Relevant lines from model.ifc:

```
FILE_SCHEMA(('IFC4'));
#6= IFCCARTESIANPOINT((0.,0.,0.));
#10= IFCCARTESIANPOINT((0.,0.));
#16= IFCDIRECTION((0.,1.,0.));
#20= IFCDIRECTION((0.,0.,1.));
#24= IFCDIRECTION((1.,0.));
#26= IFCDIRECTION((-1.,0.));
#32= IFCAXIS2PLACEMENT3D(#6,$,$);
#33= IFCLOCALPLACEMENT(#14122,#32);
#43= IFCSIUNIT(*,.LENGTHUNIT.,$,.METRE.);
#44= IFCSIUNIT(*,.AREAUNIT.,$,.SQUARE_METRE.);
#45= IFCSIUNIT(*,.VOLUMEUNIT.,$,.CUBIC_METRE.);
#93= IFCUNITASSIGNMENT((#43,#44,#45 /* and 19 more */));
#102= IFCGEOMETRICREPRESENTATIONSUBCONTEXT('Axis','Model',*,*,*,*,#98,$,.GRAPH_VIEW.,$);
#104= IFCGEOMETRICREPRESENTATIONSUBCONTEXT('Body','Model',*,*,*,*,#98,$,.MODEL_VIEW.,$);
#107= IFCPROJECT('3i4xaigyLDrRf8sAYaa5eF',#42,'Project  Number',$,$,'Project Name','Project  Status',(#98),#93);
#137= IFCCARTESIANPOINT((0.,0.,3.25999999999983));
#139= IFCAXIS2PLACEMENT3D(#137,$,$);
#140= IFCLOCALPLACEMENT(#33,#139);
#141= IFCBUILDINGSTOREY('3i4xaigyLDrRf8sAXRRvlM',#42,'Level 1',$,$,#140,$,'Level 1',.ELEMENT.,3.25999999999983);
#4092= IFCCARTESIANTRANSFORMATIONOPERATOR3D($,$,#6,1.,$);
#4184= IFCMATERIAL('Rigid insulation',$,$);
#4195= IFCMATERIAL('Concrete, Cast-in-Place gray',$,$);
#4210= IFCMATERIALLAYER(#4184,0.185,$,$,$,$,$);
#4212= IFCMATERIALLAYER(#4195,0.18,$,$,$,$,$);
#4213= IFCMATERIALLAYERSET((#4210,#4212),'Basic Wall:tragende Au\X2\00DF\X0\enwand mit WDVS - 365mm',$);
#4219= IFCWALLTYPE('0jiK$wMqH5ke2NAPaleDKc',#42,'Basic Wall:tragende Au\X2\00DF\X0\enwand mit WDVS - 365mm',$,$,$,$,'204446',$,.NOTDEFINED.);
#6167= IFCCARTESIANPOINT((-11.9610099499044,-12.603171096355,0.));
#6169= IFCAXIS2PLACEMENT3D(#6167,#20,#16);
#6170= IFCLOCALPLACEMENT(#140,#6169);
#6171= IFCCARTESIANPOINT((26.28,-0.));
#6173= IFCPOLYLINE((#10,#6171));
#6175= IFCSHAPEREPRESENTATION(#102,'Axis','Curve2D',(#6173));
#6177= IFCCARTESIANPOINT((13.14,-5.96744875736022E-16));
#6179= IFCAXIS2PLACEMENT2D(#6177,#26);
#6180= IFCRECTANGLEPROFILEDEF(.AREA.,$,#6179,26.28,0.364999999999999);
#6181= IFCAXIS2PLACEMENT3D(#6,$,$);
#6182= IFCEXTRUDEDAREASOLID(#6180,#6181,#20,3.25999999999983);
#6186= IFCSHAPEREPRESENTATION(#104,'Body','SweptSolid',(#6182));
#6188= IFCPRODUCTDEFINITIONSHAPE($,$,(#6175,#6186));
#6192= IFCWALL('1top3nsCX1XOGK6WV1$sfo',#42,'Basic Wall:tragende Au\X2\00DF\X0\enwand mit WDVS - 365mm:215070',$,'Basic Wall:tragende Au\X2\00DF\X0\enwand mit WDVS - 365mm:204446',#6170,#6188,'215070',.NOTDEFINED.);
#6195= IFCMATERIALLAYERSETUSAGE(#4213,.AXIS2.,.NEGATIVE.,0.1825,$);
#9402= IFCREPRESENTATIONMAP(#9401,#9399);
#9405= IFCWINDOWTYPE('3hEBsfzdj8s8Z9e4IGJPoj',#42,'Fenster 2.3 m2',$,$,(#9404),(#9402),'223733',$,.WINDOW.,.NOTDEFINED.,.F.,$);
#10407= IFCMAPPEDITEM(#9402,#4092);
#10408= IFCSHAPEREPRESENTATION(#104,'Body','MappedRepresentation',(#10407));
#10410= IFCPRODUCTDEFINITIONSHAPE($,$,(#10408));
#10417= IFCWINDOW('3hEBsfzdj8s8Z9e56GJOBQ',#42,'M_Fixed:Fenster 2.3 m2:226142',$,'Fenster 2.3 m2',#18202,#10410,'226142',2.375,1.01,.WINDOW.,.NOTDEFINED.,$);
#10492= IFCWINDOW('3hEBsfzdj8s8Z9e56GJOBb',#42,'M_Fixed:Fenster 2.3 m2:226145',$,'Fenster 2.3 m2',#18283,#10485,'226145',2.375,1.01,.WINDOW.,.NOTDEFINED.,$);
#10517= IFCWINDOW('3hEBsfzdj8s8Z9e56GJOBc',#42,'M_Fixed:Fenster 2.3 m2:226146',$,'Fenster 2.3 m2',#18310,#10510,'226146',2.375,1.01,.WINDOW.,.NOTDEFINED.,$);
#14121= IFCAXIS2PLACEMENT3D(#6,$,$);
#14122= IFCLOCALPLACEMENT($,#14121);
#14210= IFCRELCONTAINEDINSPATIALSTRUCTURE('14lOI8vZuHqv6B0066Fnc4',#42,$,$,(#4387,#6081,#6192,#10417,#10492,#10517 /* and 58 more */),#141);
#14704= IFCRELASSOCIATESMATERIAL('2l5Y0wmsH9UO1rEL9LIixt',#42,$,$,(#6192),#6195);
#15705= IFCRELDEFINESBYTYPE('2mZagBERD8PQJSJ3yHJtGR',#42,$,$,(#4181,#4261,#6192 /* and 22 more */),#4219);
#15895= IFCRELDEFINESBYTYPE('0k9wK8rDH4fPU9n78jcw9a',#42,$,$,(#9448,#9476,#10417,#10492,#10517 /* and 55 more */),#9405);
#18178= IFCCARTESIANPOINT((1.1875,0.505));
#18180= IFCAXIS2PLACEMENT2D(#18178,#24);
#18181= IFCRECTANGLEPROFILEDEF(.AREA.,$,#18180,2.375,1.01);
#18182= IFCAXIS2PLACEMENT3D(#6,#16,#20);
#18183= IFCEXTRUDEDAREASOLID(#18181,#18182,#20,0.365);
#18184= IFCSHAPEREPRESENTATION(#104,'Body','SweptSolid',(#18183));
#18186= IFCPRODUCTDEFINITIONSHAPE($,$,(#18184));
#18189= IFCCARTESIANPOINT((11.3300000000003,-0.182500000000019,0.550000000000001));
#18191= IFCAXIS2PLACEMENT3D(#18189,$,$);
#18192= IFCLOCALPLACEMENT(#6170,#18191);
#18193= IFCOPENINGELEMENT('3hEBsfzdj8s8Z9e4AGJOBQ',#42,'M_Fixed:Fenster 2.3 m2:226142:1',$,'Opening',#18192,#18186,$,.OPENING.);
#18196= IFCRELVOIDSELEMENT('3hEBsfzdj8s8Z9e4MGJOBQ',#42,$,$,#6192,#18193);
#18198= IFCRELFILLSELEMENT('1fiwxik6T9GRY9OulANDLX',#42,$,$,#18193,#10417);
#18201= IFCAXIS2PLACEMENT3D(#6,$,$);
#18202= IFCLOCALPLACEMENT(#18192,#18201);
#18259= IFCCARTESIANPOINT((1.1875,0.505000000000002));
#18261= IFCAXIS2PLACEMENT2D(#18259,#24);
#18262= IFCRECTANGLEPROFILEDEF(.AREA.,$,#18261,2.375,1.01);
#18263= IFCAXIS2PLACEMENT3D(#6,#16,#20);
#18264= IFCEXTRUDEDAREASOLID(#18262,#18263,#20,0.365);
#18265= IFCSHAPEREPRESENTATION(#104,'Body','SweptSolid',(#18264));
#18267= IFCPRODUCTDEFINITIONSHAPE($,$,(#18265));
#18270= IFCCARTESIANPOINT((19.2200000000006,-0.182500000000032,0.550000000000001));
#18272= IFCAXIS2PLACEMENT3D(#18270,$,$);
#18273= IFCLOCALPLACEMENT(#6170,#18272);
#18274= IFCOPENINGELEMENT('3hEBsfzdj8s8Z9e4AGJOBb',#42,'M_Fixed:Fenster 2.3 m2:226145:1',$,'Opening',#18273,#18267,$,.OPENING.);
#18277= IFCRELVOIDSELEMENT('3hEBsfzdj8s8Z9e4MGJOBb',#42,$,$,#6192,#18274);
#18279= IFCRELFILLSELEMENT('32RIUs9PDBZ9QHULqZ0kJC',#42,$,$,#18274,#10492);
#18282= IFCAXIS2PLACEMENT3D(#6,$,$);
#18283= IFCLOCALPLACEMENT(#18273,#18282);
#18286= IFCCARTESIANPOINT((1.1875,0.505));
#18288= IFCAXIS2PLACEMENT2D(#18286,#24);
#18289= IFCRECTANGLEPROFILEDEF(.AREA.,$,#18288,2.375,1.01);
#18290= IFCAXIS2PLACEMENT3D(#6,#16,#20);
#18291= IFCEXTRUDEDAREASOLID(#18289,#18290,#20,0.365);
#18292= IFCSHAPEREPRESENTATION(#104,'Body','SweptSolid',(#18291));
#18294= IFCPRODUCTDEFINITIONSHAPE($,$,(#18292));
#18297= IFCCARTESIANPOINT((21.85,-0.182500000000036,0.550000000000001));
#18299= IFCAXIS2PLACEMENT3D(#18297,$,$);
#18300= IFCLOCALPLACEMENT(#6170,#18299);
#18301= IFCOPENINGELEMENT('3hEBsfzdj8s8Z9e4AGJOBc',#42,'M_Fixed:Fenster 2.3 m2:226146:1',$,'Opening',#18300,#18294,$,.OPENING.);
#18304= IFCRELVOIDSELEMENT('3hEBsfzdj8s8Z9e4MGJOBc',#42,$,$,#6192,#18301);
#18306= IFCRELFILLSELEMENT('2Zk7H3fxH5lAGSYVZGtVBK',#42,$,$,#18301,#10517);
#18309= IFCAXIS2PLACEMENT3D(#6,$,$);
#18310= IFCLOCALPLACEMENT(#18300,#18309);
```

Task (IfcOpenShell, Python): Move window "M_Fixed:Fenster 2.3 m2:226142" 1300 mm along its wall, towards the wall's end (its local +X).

```python
import ifcopenshell
import ifcopenshell.api.geometry
import ifcopenshell.util.placement

model = ifcopenshell.open("model.ifc")

window = model.by_guid("3hEBsfzdj8s8Z9e56GJOBQ")
opening = window.FillsVoids[0].RelatingOpeningElement
wall = opening.VoidsElements[0].RelatingBuildingElement

wall_matrix = ifcopenshell.util.placement.get_local_placement(wall.ObjectPlacement)
shift = wall_matrix[:3, 0] * 1.3
before = ifcopenshell.util.placement.get_local_placement(window.ObjectPlacement)[:3, 3].copy()

# The window is placed relative to its opening, so it follows when the opening moves.
matrix = ifcopenshell.util.placement.get_local_placement(opening.ObjectPlacement)
matrix[:3, 3] += shift
ifcopenshell.api.geometry.edit_object_placement(
    model, product=opening, matrix=matrix, is_si=False, should_transform_children=True
)

after = ifcopenshell.util.placement.get_local_placement(window.ObjectPlacement)[:3, 3]
print("window moved by", (after - before).round(3) + 0.0)

model.write("model_v2.ifc")
```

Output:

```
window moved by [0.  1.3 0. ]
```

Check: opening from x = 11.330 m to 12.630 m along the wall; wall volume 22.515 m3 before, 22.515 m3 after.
